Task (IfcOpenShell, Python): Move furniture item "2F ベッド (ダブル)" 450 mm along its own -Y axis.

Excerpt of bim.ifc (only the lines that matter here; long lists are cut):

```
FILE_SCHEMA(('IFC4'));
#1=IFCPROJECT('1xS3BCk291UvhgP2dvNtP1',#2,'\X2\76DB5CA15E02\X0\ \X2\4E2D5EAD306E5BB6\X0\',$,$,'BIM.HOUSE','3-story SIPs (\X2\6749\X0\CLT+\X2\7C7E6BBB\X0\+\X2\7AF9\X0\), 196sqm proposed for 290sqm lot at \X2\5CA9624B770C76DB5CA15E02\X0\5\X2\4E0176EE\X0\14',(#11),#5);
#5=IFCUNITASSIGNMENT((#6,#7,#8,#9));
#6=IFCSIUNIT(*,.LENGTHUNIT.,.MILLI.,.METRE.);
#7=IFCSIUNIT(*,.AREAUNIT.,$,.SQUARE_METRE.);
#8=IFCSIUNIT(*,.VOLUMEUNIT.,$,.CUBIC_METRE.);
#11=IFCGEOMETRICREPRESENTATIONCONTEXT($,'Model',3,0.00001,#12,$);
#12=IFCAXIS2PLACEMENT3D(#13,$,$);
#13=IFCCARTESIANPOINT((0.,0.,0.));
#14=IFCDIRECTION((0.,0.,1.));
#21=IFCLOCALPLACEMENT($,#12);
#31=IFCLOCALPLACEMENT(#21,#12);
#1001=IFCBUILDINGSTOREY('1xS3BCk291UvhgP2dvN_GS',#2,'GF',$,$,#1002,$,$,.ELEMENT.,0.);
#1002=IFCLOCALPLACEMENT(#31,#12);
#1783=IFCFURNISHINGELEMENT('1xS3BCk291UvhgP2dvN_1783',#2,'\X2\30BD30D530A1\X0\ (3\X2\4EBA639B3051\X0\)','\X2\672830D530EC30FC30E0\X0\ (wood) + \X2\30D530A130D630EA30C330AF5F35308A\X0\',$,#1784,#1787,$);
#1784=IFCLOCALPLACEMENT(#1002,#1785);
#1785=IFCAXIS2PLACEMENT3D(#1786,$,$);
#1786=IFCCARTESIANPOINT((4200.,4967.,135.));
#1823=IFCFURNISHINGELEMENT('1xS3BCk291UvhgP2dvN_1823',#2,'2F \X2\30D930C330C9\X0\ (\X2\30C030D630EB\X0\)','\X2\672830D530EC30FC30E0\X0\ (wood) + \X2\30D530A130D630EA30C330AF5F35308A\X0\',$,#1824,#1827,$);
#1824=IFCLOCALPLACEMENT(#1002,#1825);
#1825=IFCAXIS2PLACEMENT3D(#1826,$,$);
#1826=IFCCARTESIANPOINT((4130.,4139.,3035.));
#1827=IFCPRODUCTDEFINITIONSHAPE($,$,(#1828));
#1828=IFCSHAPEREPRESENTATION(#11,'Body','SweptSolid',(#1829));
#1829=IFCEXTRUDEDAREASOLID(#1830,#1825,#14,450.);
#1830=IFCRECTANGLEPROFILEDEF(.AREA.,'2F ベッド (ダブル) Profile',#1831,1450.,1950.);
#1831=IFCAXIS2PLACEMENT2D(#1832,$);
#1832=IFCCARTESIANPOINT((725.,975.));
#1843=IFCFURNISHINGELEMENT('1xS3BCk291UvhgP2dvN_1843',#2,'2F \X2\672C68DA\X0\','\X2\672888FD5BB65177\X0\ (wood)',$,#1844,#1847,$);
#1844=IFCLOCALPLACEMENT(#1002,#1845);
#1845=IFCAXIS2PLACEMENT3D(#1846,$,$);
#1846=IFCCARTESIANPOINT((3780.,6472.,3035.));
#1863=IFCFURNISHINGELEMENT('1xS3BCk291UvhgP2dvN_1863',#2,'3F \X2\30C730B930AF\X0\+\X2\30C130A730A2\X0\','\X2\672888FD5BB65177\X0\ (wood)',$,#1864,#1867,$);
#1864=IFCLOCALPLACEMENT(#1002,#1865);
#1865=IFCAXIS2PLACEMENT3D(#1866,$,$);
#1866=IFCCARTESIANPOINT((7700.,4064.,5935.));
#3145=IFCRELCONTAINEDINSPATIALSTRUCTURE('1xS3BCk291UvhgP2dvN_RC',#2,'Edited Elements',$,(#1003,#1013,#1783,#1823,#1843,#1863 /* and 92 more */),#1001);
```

```python
import ifcopenshell
import ifcopenshell.api.geometry
import ifcopenshell.util.placement

model = ifcopenshell.open("bim.ifc")

item = model.by_guid("1xS3BCk291UvhgP2dvN_1823")
matrix = ifcopenshell.util.placement.get_local_placement(item.ObjectPlacement)
matrix[:3, 3] -= matrix[:3, 1] * 450.0
ifcopenshell.api.geometry.edit_object_placement(model, product=item, matrix=matrix, is_si=False)

print(ifcopenshell.util.placement.get_local_placement(item.ObjectPlacement).round(3) + 0.0)

model.write("bim_v2.ifc")
```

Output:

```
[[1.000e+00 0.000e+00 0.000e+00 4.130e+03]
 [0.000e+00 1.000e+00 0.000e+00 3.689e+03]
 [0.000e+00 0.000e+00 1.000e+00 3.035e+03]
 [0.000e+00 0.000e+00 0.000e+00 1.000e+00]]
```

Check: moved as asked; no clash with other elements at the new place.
